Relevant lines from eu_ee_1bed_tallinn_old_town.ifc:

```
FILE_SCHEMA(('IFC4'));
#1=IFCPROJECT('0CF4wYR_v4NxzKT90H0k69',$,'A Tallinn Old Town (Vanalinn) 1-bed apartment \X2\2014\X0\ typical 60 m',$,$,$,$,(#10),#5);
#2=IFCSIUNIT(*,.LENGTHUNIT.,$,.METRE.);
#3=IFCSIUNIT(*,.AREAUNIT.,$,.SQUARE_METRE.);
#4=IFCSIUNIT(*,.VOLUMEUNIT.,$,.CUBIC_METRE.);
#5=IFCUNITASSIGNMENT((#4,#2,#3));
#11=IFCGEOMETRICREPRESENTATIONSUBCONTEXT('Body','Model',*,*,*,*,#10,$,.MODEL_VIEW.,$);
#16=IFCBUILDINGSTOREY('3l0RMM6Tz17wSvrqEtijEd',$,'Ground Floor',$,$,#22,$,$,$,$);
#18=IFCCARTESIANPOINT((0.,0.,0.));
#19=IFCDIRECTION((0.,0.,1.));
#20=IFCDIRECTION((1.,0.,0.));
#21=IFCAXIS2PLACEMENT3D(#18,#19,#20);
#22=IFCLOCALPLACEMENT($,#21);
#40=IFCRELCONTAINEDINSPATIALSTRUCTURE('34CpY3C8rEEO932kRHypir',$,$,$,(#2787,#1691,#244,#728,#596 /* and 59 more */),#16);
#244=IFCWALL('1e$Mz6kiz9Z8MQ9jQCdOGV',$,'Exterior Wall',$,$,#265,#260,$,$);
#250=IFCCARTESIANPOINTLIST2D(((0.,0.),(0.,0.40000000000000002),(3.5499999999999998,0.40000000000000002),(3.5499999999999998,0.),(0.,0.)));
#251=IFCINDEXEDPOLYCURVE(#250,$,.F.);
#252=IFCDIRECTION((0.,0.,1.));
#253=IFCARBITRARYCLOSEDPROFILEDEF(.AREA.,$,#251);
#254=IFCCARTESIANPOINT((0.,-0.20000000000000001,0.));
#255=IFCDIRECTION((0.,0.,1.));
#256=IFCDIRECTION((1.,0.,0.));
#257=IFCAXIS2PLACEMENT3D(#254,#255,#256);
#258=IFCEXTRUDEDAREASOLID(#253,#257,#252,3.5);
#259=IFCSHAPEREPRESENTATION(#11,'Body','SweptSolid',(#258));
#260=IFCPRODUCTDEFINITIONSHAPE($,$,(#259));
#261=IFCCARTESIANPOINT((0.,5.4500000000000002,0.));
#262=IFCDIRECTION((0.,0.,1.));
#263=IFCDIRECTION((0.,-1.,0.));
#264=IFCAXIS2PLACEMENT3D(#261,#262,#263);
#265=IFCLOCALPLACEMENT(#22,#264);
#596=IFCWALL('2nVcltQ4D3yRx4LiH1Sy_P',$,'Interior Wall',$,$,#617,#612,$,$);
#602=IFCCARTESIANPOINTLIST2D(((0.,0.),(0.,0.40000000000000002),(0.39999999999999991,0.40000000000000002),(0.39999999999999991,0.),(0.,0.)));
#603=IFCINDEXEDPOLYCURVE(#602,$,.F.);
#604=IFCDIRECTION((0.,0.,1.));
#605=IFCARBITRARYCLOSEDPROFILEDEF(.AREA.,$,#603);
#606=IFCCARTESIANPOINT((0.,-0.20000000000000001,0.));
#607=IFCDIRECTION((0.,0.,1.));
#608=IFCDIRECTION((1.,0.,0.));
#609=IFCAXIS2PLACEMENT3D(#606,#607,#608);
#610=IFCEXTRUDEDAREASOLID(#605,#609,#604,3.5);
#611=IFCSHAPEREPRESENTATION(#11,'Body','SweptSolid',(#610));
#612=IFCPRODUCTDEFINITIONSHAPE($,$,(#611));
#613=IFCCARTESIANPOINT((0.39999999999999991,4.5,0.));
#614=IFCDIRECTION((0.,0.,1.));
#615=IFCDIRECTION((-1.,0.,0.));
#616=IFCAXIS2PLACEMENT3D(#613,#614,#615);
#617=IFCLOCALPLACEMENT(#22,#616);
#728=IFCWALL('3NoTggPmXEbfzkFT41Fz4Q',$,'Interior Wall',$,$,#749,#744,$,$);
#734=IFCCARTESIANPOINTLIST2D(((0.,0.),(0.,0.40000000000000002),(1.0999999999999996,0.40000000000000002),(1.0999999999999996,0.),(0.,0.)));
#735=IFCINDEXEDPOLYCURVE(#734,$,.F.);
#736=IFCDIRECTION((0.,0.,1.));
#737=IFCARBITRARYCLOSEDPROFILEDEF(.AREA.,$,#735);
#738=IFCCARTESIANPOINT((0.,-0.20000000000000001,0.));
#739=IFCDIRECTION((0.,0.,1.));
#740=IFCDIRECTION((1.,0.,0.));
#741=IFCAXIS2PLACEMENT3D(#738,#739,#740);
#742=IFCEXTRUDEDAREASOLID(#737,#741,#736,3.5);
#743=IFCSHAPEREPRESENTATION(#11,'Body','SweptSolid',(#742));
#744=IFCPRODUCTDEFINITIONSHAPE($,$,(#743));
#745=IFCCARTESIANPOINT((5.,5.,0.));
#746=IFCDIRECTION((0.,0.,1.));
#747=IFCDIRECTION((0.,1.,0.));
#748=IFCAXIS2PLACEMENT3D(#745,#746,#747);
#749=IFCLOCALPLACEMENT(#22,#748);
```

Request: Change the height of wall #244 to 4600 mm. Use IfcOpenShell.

```python
import ifcopenshell
import ifcopenshell.geom
import ifcopenshell.util.representation
import ifcopenshell.util.shape
import ifcopenshell.util.unit

model = ifcopenshell.open("eu_ee_1bed_tallinn_old_town.ifc")
unit_scale = ifcopenshell.util.unit.calculate_unit_scale(model)
settings = ifcopenshell.geom.settings()


def volume(element):
    """Net volume in cubic metres, openings subtracted."""
    shape = ifcopenshell.geom.create_shape(settings, element)
    return ifcopenshell.util.shape.get_volume(shape.geometry)


wall = model.by_guid("1e$Mz6kiz9Z8MQ9jQCdOGV")
before = volume(wall)

body = ifcopenshell.util.representation.get_representation(wall, "Model", "Body")
solid = body.Items[0]
old_height = solid.Depth
solid.Depth = 4.6 / unit_scale
after = volume(wall)

print(f"height {old_height:g} -> {solid.Depth:g}, volume {before:.3f} -> {after:.3f} m3")

model.write("eu_ee_1bed_tallinn_old_town_updated.ifc")
```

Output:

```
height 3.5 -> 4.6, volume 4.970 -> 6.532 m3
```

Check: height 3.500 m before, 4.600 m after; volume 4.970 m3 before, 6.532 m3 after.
